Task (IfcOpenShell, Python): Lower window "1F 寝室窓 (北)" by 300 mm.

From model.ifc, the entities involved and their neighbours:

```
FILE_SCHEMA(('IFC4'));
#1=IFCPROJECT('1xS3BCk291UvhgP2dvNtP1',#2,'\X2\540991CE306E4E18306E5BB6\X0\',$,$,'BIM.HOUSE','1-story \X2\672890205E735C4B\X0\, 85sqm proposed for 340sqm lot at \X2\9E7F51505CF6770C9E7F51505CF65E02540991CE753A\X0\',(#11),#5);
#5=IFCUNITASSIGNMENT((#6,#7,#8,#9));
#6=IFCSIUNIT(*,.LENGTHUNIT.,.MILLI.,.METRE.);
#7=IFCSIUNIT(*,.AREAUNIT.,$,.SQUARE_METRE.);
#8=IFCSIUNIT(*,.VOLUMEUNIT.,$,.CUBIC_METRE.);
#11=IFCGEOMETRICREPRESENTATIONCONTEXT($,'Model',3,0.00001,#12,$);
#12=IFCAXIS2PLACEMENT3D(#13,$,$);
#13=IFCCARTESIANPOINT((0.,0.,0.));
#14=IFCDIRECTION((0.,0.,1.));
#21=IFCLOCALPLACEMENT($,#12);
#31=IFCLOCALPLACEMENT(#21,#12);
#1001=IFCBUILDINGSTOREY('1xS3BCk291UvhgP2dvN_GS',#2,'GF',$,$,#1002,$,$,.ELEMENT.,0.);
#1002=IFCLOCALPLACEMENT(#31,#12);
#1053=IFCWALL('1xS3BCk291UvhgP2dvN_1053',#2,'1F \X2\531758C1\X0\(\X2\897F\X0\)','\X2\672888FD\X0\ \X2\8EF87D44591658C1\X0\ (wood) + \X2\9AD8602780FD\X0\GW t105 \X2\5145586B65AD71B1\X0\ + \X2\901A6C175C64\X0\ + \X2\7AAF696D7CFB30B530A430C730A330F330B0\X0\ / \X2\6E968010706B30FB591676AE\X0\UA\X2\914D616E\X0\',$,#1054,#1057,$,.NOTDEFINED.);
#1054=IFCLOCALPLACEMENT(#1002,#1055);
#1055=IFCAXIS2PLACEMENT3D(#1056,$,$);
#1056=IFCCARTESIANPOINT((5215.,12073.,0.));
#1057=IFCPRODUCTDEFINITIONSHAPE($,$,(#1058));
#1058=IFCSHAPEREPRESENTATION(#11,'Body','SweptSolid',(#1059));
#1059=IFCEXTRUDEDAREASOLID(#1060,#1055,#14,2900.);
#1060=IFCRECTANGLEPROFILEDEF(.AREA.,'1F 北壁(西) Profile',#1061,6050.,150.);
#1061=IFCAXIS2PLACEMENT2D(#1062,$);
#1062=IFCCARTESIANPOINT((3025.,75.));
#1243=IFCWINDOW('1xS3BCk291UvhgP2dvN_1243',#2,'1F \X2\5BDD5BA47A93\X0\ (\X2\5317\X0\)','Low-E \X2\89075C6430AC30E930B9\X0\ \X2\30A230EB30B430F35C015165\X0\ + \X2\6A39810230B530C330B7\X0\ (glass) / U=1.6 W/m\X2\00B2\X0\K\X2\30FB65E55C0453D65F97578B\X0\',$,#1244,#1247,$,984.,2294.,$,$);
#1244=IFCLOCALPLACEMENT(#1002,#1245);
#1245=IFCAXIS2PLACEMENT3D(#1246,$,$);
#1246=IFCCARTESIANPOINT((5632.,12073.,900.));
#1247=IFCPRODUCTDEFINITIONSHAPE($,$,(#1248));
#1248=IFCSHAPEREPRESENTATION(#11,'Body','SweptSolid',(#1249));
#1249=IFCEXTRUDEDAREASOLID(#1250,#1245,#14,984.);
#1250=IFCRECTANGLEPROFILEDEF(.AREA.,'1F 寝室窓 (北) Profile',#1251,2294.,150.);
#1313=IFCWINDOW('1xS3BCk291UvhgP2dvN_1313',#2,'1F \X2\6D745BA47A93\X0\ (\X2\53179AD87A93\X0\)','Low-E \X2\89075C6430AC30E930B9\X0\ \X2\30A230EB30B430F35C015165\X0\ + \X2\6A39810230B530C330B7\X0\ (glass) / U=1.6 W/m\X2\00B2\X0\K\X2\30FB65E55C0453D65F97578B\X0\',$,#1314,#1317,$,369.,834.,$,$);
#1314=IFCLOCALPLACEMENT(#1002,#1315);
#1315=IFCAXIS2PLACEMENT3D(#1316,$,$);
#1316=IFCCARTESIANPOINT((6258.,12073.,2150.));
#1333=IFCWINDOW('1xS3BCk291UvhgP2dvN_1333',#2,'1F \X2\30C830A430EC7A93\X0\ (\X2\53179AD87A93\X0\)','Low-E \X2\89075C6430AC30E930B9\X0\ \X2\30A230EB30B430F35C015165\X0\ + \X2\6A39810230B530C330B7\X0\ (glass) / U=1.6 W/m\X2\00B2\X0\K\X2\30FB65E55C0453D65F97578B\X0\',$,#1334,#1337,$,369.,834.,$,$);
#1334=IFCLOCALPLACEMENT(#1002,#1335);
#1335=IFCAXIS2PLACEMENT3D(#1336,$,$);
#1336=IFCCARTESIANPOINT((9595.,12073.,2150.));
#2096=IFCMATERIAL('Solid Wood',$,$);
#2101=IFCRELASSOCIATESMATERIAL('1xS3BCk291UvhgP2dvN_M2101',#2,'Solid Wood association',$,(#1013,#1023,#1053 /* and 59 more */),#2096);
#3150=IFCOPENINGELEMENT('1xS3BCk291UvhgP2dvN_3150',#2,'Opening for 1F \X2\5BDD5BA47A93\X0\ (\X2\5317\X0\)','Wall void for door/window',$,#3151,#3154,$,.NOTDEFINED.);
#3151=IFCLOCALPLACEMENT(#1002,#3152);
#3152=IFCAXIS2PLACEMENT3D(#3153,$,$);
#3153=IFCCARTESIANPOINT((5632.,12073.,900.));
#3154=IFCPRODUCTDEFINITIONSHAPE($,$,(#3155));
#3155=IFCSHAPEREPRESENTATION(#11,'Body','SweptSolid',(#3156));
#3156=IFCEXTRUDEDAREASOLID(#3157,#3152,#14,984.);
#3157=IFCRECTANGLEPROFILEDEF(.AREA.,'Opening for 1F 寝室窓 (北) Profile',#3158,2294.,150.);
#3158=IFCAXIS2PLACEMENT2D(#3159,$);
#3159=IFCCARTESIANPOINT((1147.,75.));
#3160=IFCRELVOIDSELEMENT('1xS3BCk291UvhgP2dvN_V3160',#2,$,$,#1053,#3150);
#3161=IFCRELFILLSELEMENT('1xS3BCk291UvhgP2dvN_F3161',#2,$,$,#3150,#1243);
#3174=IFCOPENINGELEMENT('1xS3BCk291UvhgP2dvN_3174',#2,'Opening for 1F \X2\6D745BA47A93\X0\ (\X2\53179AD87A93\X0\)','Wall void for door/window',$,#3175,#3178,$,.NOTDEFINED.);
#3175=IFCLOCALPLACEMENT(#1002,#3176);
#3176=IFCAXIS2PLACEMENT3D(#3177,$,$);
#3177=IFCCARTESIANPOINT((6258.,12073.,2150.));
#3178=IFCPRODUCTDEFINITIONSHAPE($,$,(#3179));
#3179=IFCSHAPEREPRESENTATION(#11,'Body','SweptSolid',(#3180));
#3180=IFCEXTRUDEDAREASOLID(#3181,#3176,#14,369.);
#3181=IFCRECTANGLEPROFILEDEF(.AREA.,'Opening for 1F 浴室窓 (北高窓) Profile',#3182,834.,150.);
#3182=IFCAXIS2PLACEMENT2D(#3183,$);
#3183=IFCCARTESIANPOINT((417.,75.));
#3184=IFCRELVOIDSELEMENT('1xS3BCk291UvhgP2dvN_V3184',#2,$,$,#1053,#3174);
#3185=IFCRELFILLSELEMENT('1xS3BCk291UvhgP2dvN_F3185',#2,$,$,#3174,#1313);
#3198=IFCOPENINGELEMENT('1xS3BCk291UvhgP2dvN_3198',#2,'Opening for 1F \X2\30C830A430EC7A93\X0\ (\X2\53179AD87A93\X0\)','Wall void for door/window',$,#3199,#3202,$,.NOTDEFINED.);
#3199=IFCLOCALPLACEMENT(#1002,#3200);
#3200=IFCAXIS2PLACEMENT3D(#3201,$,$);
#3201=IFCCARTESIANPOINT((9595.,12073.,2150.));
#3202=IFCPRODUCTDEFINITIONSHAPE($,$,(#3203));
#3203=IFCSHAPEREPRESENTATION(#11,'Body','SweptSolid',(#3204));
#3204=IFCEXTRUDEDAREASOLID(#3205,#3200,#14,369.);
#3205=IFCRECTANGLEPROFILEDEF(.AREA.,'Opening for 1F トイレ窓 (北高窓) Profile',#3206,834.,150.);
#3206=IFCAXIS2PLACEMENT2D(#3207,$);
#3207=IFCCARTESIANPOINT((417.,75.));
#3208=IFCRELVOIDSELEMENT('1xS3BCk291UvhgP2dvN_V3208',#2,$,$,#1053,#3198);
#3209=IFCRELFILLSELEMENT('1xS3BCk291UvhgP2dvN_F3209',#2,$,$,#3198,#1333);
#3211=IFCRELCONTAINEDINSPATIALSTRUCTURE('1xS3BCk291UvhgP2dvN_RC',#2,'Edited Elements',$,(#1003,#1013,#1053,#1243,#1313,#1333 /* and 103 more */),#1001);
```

```python
import numpy as np
import ifcopenshell
import ifcopenshell.api.geometry
import ifcopenshell.util.placement
import ifcopenshell.util.unit

model = ifcopenshell.open("model.ifc")
unit_scale = ifcopenshell.util.unit.calculate_unit_scale(model)

window = model.by_guid("1xS3BCk291UvhgP2dvN_1243")
opening = window.FillsVoids[0].RelatingOpeningElement
dz = -0.3 / unit_scale

shift = np.array([0.0, 0.0, dz])
# The window is not placed relative to its opening, so move both.
for product in (opening, window):
    matrix = ifcopenshell.util.placement.get_local_placement(product.ObjectPlacement)
    matrix[:3, 3] += shift
    ifcopenshell.api.geometry.edit_object_placement(model, product=product, matrix=matrix, is_si=False)

print(f"moved by {dz * unit_scale:+.3f} m")

model.write("model_edited.ifc")
```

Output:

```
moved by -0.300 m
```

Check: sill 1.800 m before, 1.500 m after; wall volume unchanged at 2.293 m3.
